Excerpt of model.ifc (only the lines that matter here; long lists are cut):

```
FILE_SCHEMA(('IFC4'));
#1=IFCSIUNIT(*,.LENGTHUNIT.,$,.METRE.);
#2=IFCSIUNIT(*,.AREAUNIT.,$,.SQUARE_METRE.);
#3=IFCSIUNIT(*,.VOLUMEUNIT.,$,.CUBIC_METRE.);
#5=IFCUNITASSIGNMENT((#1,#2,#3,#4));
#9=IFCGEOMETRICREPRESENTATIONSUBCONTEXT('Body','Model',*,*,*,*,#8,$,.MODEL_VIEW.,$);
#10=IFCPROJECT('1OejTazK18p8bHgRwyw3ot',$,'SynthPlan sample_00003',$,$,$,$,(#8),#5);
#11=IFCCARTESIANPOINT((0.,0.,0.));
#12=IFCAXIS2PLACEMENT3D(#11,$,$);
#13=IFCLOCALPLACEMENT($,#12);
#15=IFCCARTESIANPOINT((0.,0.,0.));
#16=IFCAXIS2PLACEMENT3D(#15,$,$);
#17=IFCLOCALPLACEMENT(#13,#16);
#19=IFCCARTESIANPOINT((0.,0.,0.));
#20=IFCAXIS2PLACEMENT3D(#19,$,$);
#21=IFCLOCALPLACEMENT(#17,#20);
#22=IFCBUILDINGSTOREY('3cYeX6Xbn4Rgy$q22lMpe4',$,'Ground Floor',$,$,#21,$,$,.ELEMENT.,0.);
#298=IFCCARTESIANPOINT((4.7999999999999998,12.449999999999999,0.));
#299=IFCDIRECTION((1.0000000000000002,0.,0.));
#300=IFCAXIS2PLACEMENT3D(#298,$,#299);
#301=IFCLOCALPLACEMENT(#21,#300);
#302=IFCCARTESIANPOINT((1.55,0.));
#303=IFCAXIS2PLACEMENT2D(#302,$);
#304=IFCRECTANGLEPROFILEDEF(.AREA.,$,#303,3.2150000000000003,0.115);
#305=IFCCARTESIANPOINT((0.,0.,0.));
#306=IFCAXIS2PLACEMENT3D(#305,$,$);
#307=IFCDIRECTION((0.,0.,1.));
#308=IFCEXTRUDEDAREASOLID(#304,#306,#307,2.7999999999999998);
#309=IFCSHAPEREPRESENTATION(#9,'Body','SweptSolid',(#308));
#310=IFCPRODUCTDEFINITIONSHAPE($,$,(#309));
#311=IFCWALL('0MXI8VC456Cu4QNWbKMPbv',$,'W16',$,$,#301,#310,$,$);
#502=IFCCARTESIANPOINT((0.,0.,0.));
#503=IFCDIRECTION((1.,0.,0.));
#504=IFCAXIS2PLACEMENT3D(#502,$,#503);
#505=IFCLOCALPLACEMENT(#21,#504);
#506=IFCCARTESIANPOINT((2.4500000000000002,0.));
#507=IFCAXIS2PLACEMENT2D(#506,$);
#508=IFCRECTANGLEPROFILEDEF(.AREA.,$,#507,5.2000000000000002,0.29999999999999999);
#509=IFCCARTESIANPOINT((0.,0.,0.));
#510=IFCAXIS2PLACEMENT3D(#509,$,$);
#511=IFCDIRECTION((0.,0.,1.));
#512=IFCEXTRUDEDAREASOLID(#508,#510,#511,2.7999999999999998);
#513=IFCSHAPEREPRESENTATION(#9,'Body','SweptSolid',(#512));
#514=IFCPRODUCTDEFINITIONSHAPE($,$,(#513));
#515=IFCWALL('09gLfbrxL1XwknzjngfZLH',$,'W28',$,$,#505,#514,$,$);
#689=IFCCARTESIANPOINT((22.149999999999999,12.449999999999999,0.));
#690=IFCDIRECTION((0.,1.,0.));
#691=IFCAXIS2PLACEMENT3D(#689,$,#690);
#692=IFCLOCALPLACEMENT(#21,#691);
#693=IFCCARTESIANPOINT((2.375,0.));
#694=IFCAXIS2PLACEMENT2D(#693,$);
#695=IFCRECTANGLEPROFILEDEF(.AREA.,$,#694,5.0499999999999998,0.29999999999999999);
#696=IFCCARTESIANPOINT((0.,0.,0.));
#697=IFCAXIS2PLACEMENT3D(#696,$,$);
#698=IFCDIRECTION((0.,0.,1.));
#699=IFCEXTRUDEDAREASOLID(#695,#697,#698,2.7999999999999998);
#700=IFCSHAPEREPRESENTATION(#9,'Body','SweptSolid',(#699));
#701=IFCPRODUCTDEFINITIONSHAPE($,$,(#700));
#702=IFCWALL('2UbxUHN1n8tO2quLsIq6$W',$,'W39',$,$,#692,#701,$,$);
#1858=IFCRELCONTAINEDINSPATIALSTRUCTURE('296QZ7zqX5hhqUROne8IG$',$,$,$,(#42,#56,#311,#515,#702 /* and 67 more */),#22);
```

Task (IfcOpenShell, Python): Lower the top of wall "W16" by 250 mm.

```python
import ifcopenshell
import ifcopenshell.geom
import ifcopenshell.util.representation
import ifcopenshell.util.shape

model = ifcopenshell.open("model.ifc")
settings = ifcopenshell.geom.settings()


def volume(element):
    """Net volume in cubic metres, openings subtracted."""
    shape = ifcopenshell.geom.create_shape(settings, element)
    return ifcopenshell.util.shape.get_volume(shape.geometry)


wall = model.by_guid("0MXI8VC456Cu4QNWbKMPbv")
before = volume(wall)

body = ifcopenshell.util.representation.get_representation(wall, "Model", "Body")
solid = body.Items[0]
old_height = solid.Depth
solid.Depth -= 0.25
after = volume(wall)

print(f"height {old_height:g} -> {solid.Depth:g}, volume {before:.3f} -> {after:.3f} m3")

model.write("model_updated.ifc")
```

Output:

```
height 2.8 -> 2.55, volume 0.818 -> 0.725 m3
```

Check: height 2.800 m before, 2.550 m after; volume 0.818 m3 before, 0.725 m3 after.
